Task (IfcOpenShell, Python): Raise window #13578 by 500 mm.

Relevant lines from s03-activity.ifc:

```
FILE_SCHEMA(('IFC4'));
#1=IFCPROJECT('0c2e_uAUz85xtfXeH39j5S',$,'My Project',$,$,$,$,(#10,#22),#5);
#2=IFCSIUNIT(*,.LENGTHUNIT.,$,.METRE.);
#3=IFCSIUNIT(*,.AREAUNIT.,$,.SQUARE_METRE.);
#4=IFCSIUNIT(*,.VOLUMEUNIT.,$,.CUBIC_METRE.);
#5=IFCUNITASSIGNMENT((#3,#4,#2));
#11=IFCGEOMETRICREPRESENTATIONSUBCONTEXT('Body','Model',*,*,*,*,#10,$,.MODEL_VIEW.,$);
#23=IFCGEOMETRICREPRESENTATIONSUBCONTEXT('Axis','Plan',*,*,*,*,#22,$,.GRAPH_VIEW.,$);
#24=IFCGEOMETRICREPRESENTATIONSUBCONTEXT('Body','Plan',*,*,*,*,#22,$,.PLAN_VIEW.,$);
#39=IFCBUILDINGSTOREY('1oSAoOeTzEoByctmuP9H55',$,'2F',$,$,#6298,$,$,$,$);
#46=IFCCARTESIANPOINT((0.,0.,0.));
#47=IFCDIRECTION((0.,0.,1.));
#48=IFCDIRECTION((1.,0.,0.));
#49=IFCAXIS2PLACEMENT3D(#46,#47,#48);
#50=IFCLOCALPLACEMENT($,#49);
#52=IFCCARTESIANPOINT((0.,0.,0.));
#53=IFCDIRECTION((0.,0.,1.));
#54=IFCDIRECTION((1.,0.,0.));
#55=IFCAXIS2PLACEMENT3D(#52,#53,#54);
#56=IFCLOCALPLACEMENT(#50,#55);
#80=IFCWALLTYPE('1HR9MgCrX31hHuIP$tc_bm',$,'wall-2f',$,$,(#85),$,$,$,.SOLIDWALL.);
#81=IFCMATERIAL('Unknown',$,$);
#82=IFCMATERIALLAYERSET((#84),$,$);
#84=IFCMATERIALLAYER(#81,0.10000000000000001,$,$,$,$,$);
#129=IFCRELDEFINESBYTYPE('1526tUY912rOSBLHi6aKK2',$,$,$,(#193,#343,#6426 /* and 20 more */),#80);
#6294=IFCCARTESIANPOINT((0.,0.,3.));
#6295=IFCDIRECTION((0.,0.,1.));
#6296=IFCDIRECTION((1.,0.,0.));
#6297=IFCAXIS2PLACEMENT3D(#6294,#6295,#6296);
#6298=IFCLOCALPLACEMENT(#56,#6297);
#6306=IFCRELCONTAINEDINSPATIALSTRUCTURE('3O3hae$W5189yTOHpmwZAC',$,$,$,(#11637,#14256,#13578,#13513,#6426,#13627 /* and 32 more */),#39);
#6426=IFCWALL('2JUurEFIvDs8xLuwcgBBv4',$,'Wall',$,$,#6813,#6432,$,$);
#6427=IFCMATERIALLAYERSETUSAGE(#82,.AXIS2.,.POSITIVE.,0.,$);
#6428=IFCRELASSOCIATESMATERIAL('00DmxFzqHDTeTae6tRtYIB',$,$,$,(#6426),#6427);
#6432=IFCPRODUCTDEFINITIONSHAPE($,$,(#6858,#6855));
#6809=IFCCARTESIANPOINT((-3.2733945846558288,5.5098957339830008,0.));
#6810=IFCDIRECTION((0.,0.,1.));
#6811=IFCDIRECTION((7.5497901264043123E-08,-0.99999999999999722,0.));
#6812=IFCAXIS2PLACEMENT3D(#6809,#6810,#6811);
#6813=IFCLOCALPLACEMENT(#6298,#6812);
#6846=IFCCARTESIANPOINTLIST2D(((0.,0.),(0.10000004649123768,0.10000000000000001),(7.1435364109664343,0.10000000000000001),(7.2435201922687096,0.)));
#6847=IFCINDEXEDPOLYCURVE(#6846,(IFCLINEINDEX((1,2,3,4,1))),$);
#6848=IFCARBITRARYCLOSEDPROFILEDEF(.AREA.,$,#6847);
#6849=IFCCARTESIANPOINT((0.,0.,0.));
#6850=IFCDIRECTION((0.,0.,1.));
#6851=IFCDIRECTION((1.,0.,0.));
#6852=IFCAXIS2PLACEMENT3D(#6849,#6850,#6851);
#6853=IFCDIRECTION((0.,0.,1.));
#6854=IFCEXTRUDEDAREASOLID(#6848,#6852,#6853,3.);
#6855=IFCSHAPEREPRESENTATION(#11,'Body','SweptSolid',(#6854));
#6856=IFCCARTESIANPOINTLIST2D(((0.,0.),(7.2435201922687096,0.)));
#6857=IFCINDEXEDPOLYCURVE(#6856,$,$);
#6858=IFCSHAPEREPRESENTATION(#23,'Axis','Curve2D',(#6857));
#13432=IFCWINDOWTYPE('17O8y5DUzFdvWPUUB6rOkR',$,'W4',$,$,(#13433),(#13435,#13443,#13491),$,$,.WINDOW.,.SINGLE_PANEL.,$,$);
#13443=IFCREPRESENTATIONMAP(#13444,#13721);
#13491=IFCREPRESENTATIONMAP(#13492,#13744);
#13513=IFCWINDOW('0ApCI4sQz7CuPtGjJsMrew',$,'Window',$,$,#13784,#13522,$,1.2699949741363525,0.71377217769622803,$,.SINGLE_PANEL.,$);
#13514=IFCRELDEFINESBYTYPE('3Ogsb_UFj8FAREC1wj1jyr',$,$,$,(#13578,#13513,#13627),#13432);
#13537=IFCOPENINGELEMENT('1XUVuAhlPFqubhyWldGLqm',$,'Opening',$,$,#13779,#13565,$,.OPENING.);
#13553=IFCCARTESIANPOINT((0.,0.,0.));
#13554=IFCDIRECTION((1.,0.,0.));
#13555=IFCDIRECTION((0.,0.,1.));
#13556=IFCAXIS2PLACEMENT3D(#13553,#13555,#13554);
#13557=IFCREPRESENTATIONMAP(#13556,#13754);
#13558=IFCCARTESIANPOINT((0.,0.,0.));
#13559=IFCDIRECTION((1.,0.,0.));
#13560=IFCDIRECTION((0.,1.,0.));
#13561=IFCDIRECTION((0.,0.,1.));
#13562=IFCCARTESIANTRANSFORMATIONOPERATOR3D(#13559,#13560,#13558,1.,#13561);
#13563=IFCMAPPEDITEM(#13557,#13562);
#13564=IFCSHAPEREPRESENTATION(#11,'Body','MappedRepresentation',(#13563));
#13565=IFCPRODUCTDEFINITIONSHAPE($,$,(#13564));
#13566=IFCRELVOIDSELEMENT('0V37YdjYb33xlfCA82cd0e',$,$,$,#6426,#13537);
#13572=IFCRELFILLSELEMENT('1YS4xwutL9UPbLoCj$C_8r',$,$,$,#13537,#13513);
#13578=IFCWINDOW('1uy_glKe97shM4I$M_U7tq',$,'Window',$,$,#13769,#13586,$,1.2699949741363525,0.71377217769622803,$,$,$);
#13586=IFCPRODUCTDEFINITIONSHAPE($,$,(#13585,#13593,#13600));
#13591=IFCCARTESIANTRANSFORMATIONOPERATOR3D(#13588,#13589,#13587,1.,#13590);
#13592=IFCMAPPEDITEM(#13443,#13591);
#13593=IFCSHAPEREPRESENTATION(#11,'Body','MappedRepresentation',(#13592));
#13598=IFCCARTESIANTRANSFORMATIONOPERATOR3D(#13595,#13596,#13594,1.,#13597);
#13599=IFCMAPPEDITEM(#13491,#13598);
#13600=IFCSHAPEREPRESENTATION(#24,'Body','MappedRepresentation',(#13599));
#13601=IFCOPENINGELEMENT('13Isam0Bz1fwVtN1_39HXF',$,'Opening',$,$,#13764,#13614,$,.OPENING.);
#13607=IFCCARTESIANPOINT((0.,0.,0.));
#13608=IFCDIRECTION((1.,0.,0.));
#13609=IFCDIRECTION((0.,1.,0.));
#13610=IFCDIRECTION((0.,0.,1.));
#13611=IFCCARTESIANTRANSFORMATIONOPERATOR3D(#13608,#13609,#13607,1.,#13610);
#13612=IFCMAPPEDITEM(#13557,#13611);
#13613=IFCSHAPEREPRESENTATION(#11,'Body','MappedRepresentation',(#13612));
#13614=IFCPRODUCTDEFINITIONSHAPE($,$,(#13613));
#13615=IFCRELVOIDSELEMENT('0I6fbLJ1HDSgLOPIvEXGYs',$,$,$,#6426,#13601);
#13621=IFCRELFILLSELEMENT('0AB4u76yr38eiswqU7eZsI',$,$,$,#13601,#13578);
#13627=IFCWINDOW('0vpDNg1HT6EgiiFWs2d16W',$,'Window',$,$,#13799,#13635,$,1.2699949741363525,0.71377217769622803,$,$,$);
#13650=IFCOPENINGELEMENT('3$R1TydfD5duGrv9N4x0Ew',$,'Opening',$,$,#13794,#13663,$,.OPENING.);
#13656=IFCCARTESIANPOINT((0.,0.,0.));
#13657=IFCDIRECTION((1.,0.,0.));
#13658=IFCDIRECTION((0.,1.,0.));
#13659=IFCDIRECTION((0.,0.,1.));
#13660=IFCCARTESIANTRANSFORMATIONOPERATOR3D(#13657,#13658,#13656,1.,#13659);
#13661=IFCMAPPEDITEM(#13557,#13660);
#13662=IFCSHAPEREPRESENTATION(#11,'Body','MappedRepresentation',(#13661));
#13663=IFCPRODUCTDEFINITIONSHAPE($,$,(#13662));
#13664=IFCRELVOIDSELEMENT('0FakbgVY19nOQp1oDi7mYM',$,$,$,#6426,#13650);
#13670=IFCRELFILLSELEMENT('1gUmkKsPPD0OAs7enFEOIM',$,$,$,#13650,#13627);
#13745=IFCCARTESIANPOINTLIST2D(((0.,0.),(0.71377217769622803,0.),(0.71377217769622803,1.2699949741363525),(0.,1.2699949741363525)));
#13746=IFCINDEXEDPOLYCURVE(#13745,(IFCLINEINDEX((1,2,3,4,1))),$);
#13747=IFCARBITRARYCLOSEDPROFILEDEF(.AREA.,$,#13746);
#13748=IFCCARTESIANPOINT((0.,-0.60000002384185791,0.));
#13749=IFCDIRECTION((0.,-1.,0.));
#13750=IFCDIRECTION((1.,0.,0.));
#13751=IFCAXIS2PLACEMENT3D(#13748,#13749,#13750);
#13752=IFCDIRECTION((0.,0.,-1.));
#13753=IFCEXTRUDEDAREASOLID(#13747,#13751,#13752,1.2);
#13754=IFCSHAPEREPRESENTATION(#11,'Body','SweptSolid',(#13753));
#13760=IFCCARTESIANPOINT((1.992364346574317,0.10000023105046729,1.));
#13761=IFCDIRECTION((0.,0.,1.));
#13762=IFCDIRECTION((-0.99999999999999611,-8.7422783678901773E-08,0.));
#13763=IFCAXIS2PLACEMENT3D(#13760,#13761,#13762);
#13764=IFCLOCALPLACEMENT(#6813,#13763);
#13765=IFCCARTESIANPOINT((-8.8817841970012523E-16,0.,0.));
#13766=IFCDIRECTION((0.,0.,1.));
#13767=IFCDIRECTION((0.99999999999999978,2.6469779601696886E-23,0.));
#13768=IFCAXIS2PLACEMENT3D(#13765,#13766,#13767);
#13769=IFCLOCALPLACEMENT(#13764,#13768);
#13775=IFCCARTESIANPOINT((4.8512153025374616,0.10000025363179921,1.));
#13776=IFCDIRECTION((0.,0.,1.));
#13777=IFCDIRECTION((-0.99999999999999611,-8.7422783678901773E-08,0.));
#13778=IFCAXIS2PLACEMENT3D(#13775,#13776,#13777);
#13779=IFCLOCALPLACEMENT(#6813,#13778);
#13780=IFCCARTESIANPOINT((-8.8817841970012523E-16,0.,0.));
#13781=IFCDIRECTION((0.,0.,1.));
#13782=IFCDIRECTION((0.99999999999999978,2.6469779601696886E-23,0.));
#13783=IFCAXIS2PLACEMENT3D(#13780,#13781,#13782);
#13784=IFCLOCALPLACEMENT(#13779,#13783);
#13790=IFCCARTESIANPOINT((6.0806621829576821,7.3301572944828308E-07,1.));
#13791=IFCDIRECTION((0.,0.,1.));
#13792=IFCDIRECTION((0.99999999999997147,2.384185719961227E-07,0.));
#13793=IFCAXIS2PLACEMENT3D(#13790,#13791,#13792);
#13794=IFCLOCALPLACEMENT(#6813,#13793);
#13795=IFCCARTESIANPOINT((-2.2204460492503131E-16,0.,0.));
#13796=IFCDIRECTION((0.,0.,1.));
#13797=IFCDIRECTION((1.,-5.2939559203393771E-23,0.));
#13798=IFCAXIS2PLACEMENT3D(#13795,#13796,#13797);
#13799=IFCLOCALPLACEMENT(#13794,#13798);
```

```python
import numpy as np
import ifcopenshell
import ifcopenshell.api.geometry
import ifcopenshell.util.placement
import ifcopenshell.util.unit

model = ifcopenshell.open("s03-activity.ifc")
unit_scale = ifcopenshell.util.unit.calculate_unit_scale(model)

window = model.by_guid("1uy_glKe97shM4I$M_U7tq")
opening = window.FillsVoids[0].RelatingOpeningElement
dz = 0.5

shift = np.array([0.0, 0.0, dz])
# The window is placed relative to its opening, so it follows when the opening moves.
matrix = ifcopenshell.util.placement.get_local_placement(opening.ObjectPlacement)
matrix[:3, 3] += shift
ifcopenshell.api.geometry.edit_object_placement(
    model, product=opening, matrix=matrix, is_si=False, should_transform_children=True
)

print(f"moved by {dz * unit_scale:+.3f} m")

model.write("s03-activity-out.ifc")
```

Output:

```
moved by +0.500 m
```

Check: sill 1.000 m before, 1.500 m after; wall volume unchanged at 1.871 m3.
